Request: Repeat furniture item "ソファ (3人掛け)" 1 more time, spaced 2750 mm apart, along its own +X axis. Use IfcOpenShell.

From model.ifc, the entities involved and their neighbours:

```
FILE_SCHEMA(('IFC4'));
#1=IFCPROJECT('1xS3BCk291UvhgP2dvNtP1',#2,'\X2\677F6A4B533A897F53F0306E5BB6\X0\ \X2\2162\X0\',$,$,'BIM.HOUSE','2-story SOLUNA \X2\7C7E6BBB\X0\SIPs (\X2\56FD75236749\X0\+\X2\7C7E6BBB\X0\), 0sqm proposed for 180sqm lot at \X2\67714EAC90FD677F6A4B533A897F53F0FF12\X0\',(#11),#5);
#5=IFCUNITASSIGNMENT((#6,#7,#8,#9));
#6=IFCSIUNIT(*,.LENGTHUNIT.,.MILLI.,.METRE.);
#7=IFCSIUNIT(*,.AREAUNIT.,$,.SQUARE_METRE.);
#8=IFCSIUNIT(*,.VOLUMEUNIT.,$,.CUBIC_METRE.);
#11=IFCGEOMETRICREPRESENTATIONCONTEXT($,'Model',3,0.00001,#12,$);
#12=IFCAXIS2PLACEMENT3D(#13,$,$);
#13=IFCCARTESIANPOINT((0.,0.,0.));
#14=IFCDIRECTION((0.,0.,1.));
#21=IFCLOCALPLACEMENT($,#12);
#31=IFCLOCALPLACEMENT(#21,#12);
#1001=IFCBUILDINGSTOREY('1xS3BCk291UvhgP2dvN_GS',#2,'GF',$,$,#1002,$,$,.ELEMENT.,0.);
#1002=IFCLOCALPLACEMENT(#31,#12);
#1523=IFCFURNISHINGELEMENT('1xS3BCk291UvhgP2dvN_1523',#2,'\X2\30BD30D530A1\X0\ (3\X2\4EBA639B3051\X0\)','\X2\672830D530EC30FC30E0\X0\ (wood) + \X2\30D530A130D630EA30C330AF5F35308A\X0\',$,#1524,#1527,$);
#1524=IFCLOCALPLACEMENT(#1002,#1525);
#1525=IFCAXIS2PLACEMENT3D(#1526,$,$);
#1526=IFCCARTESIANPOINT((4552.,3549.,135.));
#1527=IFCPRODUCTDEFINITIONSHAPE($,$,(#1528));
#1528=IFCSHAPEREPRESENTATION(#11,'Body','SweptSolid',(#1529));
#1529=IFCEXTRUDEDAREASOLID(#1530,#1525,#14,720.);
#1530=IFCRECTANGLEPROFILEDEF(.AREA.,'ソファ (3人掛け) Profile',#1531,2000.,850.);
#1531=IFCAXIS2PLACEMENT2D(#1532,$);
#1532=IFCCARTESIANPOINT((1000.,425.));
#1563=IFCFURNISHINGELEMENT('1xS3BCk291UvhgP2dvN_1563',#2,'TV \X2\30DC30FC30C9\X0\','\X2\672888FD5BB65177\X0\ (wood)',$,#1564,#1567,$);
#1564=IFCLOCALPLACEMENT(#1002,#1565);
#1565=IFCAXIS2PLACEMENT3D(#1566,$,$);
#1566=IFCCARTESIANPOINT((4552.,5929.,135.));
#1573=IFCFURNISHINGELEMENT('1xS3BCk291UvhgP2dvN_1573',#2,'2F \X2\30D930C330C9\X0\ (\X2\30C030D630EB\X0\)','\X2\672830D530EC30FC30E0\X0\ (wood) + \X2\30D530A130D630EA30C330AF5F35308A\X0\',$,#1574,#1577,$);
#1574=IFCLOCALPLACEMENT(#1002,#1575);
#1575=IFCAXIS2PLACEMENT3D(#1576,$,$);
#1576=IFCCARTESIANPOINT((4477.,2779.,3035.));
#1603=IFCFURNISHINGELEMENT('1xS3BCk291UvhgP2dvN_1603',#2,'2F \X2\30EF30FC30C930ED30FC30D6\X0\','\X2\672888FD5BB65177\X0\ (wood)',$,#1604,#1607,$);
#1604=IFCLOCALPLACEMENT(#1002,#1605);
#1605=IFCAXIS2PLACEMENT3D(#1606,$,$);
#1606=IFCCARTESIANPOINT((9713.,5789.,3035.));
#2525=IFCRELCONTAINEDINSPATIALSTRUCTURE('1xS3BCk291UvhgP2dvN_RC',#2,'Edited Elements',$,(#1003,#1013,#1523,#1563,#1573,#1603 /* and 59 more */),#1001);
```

```python
import ifcopenshell
import ifcopenshell.api.geometry
import ifcopenshell.api.root
import ifcopenshell.util.element
import ifcopenshell.util.placement
import ifcopenshell.util.unit

model = ifcopenshell.open("model.ifc")
unit_scale = ifcopenshell.util.unit.calculate_unit_scale(model)


def reuse_history(source, copy):
    """copy_class also copies each property set's owner history, people and application; keep the originals."""
    for rel in copy.IsDefinedBy:
        if rel.is_a("IfcRelDefinesByProperties") and (history := rel.RelatingPropertyDefinition.OwnerHistory):
            rel.RelatingPropertyDefinition.OwnerHistory = source.OwnerHistory
            ifcopenshell.util.element.remove_deep2(model, history)


source = model.by_guid("1xS3BCk291UvhgP2dvN_1523")
base = ifcopenshell.util.placement.get_local_placement(source.ObjectPlacement)
step = base[:3, 0] * 2.75 / unit_scale

for i in range(1, 2):
    copy = ifcopenshell.api.root.copy_class(model, product=source)
    copy.Representation = ifcopenshell.util.element.copy_deep(
        model, source.Representation, exclude=["IfcGeometricRepresentationContext", "IfcRepresentationMap"]
    )
    reuse_history(source, copy)
    matrix = base.copy()
    matrix[:3, 3] += i * step
    print("added at", matrix[:3, 3].round(3) + 0.0)
    ifcopenshell.api.geometry.edit_object_placement(model, product=copy, matrix=matrix, is_si=False)

model.write("model_v2.ifc")
```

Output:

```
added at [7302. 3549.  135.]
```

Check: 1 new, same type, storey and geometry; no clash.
